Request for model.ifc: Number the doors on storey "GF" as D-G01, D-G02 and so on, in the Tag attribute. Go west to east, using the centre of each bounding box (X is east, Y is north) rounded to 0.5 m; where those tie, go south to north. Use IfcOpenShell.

First a look at what the model holds.

```python
import ifcopenshell
import ifcopenshell.util.element
import ifcopenshell.util.placement

model = ifcopenshell.open("model.ifc")
print(model.schema)
storey = next(s for s in model.by_type("IfcBuildingStorey") if s.Name == "GF")
doors = [e for e in ifcopenshell.util.element.get_decomposition(storey) if e.is_a("IfcDoor")]
for e in sorted(doors, key=lambda e: e.id()):
    origin = ifcopenshell.util.placement.get_local_placement(e.ObjectPlacement)[:3, 3]
    print(e.id(), e.Tag, e.Name, origin.round(2) + 0.0, sep=" | ")
```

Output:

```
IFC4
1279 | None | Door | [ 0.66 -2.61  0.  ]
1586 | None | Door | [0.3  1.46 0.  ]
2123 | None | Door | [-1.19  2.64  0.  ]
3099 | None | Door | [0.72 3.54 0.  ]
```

```python
import ifcopenshell
import ifcopenshell.geom
import ifcopenshell.util.element
import ifcopenshell.util.shape

model = ifcopenshell.open("model.ifc")
settings = ifcopenshell.geom.settings()
settings.set("use-world-coords", True)


def centre(element):
    shape = ifcopenshell.geom.create_shape(settings, element)
    return ifcopenshell.util.shape.get_bbox_centroid(shape.geometry)


storey = next(s for s in model.by_type("IfcBuildingStorey") if s.Name == "GF")
doors = [e for e in ifcopenshell.util.element.get_decomposition(storey) if e.is_a("IfcDoor")]

# Insertion points can sit at a corner or the storey origin, so sort by the geometry (in metres).
centres = {e: centre(e) for e in doors}
doors.sort(key=lambda e: (round(centres[e][0] / 0.5), centres[e][1]))

for i, e in enumerate(doors, start=1):
    number = f"D-G{i:02d}"
    e.Tag = number
    print(e.id(), number)

model.write("model_v2.ifc")
```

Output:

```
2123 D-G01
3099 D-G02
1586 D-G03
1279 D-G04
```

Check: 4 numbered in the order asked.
